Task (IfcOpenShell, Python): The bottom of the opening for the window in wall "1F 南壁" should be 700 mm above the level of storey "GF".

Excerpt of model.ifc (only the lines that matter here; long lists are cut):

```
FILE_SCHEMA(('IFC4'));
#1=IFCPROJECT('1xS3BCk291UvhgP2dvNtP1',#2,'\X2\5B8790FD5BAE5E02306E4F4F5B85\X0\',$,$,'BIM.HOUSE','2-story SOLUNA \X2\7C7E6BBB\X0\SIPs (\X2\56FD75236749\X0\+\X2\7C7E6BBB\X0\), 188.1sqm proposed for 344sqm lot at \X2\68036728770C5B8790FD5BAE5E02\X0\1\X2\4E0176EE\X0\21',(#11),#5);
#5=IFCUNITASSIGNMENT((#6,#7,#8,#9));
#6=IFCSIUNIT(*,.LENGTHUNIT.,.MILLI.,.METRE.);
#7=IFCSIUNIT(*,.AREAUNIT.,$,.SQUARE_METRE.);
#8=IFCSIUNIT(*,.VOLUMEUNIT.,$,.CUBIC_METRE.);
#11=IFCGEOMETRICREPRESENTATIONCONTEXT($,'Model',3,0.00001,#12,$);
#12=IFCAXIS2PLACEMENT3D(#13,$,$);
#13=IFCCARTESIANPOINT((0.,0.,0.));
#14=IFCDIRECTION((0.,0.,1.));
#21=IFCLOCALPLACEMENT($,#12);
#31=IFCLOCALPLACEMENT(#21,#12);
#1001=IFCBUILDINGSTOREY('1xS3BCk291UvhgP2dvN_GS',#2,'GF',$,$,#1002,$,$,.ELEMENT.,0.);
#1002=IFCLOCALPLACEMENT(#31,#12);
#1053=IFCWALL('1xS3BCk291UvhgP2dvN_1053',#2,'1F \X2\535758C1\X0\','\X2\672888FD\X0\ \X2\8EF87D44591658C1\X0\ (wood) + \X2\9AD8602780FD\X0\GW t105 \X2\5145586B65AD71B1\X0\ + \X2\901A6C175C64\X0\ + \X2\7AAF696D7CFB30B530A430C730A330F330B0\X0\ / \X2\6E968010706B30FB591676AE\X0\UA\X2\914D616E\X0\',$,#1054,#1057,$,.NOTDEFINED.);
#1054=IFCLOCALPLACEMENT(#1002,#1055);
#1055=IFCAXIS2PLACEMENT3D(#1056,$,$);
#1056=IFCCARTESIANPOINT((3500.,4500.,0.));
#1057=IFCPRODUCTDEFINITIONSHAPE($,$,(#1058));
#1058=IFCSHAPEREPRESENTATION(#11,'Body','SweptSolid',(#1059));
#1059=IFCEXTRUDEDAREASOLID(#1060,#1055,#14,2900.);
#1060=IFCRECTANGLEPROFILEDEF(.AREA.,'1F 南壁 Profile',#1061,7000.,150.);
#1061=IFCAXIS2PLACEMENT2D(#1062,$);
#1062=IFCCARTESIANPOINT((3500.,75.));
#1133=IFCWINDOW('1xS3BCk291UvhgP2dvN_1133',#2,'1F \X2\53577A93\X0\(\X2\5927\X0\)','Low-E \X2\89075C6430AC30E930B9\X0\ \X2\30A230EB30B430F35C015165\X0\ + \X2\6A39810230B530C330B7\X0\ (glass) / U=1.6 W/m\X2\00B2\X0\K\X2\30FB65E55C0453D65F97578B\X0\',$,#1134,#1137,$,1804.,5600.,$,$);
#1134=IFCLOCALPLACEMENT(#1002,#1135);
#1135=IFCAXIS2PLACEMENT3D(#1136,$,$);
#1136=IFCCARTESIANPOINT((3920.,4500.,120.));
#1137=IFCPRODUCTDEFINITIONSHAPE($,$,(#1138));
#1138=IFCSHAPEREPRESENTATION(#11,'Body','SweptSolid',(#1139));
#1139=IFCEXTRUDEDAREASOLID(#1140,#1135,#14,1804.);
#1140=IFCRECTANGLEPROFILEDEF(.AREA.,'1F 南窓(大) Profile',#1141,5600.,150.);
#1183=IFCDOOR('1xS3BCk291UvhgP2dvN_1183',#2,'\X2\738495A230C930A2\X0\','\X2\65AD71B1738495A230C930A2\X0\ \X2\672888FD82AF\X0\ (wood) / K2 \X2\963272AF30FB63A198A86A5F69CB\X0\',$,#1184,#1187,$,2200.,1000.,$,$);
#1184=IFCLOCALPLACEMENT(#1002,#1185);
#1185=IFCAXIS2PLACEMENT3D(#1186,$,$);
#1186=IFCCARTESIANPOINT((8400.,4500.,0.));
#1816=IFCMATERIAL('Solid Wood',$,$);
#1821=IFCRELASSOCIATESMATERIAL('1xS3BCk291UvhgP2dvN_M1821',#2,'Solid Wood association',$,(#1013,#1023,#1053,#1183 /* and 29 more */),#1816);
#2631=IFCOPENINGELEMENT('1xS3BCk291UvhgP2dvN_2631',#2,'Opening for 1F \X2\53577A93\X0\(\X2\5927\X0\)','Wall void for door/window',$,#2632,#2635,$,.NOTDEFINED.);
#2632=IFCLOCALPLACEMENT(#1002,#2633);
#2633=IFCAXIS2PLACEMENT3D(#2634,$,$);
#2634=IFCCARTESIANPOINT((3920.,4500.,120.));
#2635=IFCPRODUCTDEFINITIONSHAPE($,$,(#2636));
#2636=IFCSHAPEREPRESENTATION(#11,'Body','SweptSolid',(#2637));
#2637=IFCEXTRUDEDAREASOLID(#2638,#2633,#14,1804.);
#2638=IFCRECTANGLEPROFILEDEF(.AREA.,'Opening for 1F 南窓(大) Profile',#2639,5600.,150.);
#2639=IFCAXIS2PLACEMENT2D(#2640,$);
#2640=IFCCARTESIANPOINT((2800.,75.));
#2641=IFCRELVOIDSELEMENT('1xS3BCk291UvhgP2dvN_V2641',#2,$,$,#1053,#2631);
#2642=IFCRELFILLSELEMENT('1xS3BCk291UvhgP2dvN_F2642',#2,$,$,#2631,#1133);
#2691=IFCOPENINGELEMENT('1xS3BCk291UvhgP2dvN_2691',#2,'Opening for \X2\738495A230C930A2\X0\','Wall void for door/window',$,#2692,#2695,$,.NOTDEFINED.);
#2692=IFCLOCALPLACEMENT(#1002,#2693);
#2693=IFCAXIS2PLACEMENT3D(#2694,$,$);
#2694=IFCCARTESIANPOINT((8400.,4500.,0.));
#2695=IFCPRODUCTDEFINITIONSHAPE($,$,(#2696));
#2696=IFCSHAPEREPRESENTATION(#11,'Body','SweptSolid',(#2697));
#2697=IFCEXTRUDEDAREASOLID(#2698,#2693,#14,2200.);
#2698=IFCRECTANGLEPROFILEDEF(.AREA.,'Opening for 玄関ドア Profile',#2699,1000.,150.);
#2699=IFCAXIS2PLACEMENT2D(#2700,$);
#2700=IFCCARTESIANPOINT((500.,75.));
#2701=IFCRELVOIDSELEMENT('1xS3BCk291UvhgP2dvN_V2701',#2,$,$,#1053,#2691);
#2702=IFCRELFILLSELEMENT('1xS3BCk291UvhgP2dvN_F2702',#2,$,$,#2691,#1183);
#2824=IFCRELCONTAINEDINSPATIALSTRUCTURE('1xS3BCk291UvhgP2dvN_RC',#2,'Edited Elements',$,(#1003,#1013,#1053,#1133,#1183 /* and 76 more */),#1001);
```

```python
import numpy as np
import ifcopenshell
import ifcopenshell.api.geometry
import ifcopenshell.geom
import ifcopenshell.util.element
import ifcopenshell.util.placement
import ifcopenshell.util.shape
import ifcopenshell.util.unit

model = ifcopenshell.open("model.ifc")
unit_scale = ifcopenshell.util.unit.calculate_unit_scale(model)

window = model.by_guid("1xS3BCk291UvhgP2dvN_1133")
opening = window.FillsVoids[0].RelatingOpeningElement
storey = ifcopenshell.util.element.get_container(window, ifc_class="IfcBuildingStorey")
level = ifcopenshell.util.placement.get_local_placement(storey.ObjectPlacement)[2, 3]

# The opening's origin need not be at the sill, so measure its lowest point.
shape = ifcopenshell.geom.create_shape(ifcopenshell.geom.settings(), opening)
bottom = ifcopenshell.util.shape.get_shape_bottom_elevation(shape, shape.geometry) / unit_scale
dz = level + 0.7 / unit_scale - bottom

shift = np.array([0.0, 0.0, dz])
# The window is not placed relative to its opening, so move both.
for product in (opening, window):
    matrix = ifcopenshell.util.placement.get_local_placement(product.ObjectPlacement)
    matrix[:3, 3] += shift
    ifcopenshell.api.geometry.edit_object_placement(model, product=product, matrix=matrix, is_si=False)

print(f"moved by {dz * unit_scale:+.3f} m")

model.write("model_edited.ifc")
```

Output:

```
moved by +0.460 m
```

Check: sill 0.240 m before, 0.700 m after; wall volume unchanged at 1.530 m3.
